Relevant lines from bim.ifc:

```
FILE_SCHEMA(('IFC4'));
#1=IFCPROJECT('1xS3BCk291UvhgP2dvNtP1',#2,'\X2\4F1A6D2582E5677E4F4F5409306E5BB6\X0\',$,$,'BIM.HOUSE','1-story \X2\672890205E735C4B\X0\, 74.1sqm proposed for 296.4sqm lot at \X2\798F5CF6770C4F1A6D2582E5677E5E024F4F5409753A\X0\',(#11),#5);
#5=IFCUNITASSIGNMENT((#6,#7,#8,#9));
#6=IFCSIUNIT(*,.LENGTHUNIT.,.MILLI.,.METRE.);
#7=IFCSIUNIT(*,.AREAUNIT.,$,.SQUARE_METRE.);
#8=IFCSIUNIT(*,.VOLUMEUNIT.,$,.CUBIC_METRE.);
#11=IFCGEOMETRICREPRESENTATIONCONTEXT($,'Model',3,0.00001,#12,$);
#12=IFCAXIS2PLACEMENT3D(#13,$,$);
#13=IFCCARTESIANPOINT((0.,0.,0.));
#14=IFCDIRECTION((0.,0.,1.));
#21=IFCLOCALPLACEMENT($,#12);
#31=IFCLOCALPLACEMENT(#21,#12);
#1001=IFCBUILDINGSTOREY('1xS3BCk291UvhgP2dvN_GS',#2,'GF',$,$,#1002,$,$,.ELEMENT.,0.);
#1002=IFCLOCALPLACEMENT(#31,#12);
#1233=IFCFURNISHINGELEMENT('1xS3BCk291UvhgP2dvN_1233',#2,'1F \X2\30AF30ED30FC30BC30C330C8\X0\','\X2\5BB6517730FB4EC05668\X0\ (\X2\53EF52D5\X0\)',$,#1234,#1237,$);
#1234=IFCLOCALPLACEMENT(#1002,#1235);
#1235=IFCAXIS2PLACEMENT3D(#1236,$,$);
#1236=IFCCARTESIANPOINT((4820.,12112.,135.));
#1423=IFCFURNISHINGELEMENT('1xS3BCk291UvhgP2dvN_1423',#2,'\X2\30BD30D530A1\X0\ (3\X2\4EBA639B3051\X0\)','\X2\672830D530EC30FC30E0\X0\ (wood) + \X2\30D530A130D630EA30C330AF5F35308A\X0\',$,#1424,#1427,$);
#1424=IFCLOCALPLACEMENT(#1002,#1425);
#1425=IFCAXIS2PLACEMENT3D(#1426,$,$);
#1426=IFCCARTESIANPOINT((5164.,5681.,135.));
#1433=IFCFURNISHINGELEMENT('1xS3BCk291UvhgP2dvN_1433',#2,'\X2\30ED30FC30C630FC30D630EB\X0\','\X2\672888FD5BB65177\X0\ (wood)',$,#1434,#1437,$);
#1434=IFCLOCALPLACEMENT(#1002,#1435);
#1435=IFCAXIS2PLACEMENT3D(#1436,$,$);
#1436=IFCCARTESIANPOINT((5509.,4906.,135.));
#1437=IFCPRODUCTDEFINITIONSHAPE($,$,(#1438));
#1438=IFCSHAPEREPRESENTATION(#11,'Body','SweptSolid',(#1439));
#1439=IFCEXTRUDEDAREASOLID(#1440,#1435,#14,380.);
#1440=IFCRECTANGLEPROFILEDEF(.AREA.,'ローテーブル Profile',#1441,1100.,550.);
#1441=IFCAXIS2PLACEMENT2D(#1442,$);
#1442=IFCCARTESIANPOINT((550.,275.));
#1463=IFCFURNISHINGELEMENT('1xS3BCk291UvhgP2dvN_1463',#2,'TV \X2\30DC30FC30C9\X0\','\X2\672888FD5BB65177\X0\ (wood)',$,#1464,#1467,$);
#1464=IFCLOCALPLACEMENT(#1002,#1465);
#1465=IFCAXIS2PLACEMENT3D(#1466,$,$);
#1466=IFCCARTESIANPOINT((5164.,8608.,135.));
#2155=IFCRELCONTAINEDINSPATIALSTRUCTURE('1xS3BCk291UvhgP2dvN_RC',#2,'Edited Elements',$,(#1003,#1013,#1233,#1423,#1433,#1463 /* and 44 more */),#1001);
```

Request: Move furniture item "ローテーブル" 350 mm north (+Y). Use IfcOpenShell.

```python
import ifcopenshell
import ifcopenshell.api.geometry
import ifcopenshell.util.placement
import ifcopenshell.util.unit

model = ifcopenshell.open("bim.ifc")
unit_scale = ifcopenshell.util.unit.calculate_unit_scale(model)

item = model.by_guid("1xS3BCk291UvhgP2dvN_1433")
matrix = ifcopenshell.util.placement.get_local_placement(item.ObjectPlacement)
matrix[1, 3] += 0.35 / unit_scale
ifcopenshell.api.geometry.edit_object_placement(model, product=item, matrix=matrix, is_si=False)

print(ifcopenshell.util.placement.get_local_placement(item.ObjectPlacement).round(3) + 0.0)

model.write("bim-out.ifc")
```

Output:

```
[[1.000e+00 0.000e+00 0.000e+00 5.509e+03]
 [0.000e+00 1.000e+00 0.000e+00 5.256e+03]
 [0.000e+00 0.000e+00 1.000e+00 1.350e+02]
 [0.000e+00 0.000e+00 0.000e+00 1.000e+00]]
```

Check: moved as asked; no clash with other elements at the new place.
